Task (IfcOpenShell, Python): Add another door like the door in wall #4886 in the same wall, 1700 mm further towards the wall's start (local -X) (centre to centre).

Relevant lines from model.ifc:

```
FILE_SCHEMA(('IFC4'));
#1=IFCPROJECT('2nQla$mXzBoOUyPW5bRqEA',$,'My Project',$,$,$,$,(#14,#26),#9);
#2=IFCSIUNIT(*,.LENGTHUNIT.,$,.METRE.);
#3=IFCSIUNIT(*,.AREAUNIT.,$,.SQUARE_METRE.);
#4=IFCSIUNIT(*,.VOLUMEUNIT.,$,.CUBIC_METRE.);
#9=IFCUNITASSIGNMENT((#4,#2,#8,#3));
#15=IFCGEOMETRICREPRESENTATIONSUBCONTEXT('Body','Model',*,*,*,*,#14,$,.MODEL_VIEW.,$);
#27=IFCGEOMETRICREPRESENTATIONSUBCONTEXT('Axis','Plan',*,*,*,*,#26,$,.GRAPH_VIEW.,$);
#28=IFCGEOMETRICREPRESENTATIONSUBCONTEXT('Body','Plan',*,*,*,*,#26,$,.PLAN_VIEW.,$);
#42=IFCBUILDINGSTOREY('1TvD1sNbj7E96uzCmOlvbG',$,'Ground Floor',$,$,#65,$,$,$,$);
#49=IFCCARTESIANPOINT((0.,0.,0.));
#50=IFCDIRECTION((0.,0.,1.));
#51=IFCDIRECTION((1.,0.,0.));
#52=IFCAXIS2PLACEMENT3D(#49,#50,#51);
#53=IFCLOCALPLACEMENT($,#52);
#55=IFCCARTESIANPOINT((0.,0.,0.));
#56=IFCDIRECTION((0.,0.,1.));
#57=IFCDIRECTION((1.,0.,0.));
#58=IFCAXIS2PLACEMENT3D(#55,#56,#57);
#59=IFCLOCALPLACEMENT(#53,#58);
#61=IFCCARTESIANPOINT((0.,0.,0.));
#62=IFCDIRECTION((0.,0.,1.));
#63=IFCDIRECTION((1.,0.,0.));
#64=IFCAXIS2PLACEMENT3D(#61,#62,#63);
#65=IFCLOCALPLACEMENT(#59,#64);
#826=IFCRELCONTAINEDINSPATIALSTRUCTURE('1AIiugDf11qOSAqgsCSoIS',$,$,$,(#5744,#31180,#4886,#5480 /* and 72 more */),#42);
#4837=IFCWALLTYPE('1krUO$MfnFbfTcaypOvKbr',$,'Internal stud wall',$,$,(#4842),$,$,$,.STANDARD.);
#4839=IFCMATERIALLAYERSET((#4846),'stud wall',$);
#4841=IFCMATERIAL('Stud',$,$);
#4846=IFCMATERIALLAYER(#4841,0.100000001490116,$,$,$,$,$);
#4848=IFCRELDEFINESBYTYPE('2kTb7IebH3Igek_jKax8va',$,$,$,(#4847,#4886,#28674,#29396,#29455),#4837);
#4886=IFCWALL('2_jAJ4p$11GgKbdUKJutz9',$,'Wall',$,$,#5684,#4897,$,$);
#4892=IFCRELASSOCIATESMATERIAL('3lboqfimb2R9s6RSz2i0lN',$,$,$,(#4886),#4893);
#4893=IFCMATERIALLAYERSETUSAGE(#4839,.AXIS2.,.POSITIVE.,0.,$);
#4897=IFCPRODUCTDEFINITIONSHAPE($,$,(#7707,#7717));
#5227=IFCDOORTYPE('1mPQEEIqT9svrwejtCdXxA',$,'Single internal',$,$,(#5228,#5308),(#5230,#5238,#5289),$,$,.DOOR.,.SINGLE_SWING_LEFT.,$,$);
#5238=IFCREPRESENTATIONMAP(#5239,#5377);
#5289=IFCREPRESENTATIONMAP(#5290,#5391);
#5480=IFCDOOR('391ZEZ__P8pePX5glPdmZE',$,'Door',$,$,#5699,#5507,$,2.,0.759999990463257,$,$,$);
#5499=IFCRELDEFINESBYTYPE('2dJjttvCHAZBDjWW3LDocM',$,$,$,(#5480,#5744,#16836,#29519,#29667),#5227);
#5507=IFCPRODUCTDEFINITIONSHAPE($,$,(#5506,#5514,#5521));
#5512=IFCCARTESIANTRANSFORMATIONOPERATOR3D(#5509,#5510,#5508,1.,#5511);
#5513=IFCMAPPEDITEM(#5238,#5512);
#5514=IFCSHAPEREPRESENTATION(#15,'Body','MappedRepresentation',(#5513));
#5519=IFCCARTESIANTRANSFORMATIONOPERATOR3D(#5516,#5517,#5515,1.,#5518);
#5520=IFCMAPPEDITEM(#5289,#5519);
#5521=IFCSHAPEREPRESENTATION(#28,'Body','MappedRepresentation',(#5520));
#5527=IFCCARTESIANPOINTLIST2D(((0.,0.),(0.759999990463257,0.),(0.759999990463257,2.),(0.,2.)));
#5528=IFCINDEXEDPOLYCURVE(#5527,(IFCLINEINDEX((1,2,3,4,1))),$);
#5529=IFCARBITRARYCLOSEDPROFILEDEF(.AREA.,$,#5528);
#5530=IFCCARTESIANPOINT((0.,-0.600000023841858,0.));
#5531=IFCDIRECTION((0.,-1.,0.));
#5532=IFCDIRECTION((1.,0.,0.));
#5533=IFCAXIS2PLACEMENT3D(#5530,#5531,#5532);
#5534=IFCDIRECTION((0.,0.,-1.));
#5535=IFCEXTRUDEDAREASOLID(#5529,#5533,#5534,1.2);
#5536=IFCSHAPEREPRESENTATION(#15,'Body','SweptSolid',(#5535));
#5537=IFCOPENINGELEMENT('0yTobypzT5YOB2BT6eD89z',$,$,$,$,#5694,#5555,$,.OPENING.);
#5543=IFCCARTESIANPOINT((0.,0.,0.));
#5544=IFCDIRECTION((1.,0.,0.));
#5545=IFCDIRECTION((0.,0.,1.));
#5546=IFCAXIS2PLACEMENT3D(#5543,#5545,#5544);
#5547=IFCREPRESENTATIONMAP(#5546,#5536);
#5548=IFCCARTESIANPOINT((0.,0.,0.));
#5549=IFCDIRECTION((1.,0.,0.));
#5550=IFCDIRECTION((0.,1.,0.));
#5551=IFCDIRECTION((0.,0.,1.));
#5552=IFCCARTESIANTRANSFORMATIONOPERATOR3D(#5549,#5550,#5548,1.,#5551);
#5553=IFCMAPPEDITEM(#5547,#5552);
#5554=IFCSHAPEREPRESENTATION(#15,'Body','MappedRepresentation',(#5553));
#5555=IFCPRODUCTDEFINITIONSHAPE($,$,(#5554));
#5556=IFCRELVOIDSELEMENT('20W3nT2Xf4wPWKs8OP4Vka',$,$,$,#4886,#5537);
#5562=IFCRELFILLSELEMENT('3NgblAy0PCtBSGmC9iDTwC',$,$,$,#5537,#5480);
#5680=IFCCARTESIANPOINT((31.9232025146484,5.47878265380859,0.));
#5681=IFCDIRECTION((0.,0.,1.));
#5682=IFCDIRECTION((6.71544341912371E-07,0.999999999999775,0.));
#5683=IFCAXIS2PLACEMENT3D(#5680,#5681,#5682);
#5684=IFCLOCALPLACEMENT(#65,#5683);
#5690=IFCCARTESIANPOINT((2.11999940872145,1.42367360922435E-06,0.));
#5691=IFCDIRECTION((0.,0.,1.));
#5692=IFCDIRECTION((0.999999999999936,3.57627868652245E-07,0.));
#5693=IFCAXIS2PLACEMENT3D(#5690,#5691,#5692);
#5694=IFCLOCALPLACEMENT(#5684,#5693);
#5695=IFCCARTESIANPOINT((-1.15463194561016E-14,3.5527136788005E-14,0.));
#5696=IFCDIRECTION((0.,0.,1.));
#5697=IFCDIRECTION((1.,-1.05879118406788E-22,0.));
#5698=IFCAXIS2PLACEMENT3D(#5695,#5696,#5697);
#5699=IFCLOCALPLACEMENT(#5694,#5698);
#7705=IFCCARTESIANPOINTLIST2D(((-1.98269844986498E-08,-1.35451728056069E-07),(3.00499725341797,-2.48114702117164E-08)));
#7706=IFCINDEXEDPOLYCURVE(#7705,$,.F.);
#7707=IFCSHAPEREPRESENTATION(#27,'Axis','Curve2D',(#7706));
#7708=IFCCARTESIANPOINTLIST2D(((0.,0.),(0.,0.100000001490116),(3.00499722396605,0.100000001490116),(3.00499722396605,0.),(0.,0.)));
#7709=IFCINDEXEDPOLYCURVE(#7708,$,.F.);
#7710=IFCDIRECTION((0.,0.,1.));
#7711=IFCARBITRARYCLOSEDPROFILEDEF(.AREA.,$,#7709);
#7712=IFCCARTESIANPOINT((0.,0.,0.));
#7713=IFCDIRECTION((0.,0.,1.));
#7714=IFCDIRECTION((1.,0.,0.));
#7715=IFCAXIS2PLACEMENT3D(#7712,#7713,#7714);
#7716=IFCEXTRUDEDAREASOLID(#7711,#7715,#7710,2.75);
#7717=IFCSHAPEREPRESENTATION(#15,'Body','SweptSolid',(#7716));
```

```python
import ifcopenshell
import ifcopenshell.api.feature
import ifcopenshell.api.geometry
import ifcopenshell.api.root
import ifcopenshell.geom
import ifcopenshell.util.element
import ifcopenshell.util.placement
import ifcopenshell.util.shape

model = ifcopenshell.open("model.ifc")
settings = ifcopenshell.geom.settings()


def volume(element):
    """Net volume in cubic metres, openings subtracted."""
    shape = ifcopenshell.geom.create_shape(settings, element)
    return ifcopenshell.util.shape.get_volume(shape.geometry)


door = model.by_guid("391ZEZ__P8pePX5glPdmZE")
opening = door.FillsVoids[0].RelatingOpeningElement
wall = opening.VoidsElements[0].RelatingBuildingElement
before = volume(wall)
shift = ifcopenshell.util.placement.get_local_placement(wall.ObjectPlacement)[:3, 0] * -1.7

# copy_class copies the void relationship, type, container and properties, but no geometry.
new_opening = ifcopenshell.api.root.copy_class(model, product=opening)
new_opening.Representation = ifcopenshell.util.element.copy_deep(
    model, opening.Representation, exclude=["IfcGeometricRepresentationContext", "IfcRepresentationMap"]
)
new_door = ifcopenshell.api.root.copy_class(model, product=door)
new_door.Representation = ifcopenshell.util.element.copy_deep(
    model, door.Representation, exclude=["IfcGeometricRepresentationContext", "IfcRepresentationMap"]
)
ifcopenshell.api.feature.add_filling(model, opening=new_opening, element=new_door)

for old, new in ((opening, new_opening), (door, new_door)):
    matrix = ifcopenshell.util.placement.get_local_placement(old.ObjectPlacement)
    matrix[:3, 3] += shift
    ifcopenshell.api.geometry.edit_object_placement(model, product=new, matrix=matrix, is_si=False)

after = volume(wall)

print(f"wall volume {before:.3f} -> {after:.3f} m3")

model.write("model_updated.ifc")
```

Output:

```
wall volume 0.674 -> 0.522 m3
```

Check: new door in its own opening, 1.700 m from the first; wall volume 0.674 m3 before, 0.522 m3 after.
